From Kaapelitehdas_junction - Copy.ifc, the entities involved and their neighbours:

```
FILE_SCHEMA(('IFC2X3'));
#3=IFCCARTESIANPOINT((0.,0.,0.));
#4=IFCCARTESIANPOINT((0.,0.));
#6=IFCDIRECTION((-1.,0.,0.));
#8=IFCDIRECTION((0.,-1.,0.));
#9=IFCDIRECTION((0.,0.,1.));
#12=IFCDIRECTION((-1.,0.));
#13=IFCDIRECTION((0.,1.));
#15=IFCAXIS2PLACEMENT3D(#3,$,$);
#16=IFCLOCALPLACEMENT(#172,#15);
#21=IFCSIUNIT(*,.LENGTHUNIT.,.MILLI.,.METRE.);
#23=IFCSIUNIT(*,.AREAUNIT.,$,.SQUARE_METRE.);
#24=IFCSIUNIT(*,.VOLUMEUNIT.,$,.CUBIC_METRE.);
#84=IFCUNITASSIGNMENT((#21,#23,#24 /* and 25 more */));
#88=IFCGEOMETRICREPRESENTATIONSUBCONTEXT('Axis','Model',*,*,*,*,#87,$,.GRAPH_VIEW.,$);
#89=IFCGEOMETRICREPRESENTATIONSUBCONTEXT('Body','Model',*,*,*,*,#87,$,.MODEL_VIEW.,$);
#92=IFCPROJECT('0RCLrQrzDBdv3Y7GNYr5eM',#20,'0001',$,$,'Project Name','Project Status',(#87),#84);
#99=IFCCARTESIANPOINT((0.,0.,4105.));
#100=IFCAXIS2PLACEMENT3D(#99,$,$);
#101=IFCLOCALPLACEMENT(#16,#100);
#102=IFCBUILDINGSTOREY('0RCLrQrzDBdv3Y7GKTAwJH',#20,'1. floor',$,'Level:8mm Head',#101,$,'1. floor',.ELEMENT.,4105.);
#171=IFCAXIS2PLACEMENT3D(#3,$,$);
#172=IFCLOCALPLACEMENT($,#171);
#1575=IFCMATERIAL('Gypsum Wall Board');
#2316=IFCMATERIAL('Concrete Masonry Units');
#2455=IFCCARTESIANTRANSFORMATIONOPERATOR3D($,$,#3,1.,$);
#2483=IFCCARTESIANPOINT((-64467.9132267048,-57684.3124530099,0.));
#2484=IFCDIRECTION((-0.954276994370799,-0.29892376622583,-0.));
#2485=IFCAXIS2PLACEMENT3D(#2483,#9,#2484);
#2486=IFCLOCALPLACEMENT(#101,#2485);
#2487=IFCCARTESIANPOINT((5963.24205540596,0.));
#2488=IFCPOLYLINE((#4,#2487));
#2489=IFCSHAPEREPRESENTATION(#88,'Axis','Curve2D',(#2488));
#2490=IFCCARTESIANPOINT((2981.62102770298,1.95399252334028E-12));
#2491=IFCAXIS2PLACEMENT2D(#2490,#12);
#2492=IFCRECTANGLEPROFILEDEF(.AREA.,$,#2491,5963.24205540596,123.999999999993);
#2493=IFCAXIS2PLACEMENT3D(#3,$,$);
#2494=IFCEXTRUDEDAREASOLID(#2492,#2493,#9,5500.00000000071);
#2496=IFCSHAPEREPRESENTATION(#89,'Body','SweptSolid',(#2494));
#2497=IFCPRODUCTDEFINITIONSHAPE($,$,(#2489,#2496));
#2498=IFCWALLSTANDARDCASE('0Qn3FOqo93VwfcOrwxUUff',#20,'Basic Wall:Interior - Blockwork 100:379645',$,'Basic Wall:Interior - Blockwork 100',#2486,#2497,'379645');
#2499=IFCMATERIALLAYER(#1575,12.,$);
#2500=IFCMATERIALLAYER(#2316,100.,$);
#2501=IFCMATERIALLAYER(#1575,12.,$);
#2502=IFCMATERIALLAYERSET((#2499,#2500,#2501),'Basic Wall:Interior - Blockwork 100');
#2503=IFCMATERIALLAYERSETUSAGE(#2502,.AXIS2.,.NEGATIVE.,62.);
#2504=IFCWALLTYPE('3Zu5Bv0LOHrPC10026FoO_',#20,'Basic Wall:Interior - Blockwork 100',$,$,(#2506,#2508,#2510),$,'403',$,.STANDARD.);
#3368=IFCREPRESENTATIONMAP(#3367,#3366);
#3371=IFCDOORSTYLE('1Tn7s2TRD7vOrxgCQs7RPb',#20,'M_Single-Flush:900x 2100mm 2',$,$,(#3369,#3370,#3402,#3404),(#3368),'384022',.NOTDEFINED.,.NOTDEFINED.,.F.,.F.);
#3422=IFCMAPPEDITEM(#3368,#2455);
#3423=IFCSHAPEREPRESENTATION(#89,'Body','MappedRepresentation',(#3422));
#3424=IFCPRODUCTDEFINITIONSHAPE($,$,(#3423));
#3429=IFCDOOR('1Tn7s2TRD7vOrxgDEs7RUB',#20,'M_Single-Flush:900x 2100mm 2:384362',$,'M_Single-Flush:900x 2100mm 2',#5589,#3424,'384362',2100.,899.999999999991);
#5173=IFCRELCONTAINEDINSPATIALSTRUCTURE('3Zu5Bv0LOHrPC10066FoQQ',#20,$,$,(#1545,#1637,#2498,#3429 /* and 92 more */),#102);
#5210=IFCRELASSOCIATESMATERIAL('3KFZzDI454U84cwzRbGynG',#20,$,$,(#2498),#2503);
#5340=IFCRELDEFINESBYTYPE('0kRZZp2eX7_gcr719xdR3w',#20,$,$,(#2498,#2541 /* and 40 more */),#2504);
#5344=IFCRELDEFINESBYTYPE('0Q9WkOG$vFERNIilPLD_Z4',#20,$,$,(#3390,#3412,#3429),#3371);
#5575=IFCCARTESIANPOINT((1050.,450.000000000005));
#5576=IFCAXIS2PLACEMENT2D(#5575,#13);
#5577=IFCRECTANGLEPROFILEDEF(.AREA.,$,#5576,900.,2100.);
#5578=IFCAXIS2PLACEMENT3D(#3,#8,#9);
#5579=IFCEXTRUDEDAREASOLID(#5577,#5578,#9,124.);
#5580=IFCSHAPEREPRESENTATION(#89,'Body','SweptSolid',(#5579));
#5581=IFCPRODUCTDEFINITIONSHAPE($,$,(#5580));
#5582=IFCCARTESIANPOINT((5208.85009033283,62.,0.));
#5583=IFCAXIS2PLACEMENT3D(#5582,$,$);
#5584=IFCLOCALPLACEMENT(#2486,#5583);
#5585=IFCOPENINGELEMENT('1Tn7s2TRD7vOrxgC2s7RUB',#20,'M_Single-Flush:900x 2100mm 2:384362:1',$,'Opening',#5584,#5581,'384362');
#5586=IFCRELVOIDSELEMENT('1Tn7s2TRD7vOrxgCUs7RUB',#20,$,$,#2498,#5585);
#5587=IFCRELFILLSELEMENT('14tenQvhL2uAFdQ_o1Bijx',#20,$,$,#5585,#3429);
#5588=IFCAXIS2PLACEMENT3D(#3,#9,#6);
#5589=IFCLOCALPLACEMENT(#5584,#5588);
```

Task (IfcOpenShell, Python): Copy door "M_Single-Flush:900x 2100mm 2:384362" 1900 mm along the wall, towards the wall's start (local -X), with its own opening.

```python
import ifcopenshell
import ifcopenshell.api.feature
import ifcopenshell.api.geometry
import ifcopenshell.api.root
import ifcopenshell.geom
import ifcopenshell.util.element
import ifcopenshell.util.placement
import ifcopenshell.util.shape
import ifcopenshell.util.unit

model = ifcopenshell.open("Kaapelitehdas_junction - Copy.ifc")
unit_scale = ifcopenshell.util.unit.calculate_unit_scale(model)
settings = ifcopenshell.geom.settings()


def volume(element):
    """Net volume in cubic metres, openings subtracted."""
    shape = ifcopenshell.geom.create_shape(settings, element)
    return ifcopenshell.util.shape.get_volume(shape.geometry)


def reuse_history(source, copy):
    """copy_class also copies each property set's owner history, people and application; keep the originals."""
    for rel in copy.IsDefinedBy:
        if rel.is_a("IfcRelDefinesByProperties") and (history := rel.RelatingPropertyDefinition.OwnerHistory):
            rel.RelatingPropertyDefinition.OwnerHistory = source.OwnerHistory
            ifcopenshell.util.element.remove_deep2(model, history)


door = model.by_guid("1Tn7s2TRD7vOrxgDEs7RUB")
opening = door.FillsVoids[0].RelatingOpeningElement
wall = opening.VoidsElements[0].RelatingBuildingElement
before = volume(wall)
shift = ifcopenshell.util.placement.get_local_placement(wall.ObjectPlacement)[:3, 0] * -1.9 / unit_scale

# copy_class copies the void relationship, type, container and properties, but no geometry.
new_opening = ifcopenshell.api.root.copy_class(model, product=opening)
new_opening.Representation = ifcopenshell.util.element.copy_deep(
    model, opening.Representation, exclude=["IfcGeometricRepresentationContext", "IfcRepresentationMap"]
)
new_opening.Name = "M_Single-Flush:900x 2100mm 2"
new_opening.Tag = None
new_door = ifcopenshell.api.root.copy_class(model, product=door)
new_door.Representation = ifcopenshell.util.element.copy_deep(
    model, door.Representation, exclude=["IfcGeometricRepresentationContext", "IfcRepresentationMap"]
)
new_door.Name = "M_Single-Flush:900x 2100mm 2"
new_door.Tag = None
reuse_history(door, new_door)
fills = ifcopenshell.api.feature.add_filling(model, opening=new_opening, element=new_door)
fills.OwnerHistory = new_door.OwnerHistory  # required in IFC2X3

for old, new in ((opening, new_opening), (door, new_door)):
    matrix = ifcopenshell.util.placement.get_local_placement(old.ObjectPlacement)
    matrix[:3, 3] += shift
    ifcopenshell.api.geometry.edit_object_placement(model, product=new, matrix=matrix, is_si=False)

after = volume(wall)

print(f"wall volume {before:.3f} -> {after:.3f} m3")

model.write("Kaapelitehdas_junction - Copy-out.ifc")
```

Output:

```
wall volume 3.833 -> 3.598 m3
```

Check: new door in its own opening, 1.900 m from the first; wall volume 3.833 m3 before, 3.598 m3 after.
